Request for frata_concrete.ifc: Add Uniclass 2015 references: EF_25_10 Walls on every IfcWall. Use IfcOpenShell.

First a look at what the model holds.

```python
import ifcopenshell

model = ifcopenshell.open("frata_concrete.ifc")
print(model.schema)
print("classifications:", [c.Name for c in model.by_type("IfcClassification")])
for ifc_class in ("IfcDoor", "IfcRoof", "IfcStair", "IfcWall", "IfcWindow"):
    print(ifc_class, len(model.by_type(ifc_class)))
```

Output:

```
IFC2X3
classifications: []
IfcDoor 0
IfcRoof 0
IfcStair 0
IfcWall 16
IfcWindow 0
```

```python
import ifcopenshell
import ifcopenshell.api.classification

model = ifcopenshell.open("frata_concrete.ifc")

# IFC2X3 requires Source and Edition and has no link from the project to the system.
system = model.create_entity("IfcClassification", Source="NBS", Edition="2015", Name="Uniclass 2015")

codes = {
    "IfcWall": ("EF_25_10", "Walls"),
}
for ifc_class, (code, name) in codes.items():
    products = model.by_type(ifc_class)
    ifcopenshell.api.classification.add_reference(
        model, products=products, classification=system, identification=code, name=name
    )
    print(code, len(products))

model.write("frata_concrete_edited.ifc")
```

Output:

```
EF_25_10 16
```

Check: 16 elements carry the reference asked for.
